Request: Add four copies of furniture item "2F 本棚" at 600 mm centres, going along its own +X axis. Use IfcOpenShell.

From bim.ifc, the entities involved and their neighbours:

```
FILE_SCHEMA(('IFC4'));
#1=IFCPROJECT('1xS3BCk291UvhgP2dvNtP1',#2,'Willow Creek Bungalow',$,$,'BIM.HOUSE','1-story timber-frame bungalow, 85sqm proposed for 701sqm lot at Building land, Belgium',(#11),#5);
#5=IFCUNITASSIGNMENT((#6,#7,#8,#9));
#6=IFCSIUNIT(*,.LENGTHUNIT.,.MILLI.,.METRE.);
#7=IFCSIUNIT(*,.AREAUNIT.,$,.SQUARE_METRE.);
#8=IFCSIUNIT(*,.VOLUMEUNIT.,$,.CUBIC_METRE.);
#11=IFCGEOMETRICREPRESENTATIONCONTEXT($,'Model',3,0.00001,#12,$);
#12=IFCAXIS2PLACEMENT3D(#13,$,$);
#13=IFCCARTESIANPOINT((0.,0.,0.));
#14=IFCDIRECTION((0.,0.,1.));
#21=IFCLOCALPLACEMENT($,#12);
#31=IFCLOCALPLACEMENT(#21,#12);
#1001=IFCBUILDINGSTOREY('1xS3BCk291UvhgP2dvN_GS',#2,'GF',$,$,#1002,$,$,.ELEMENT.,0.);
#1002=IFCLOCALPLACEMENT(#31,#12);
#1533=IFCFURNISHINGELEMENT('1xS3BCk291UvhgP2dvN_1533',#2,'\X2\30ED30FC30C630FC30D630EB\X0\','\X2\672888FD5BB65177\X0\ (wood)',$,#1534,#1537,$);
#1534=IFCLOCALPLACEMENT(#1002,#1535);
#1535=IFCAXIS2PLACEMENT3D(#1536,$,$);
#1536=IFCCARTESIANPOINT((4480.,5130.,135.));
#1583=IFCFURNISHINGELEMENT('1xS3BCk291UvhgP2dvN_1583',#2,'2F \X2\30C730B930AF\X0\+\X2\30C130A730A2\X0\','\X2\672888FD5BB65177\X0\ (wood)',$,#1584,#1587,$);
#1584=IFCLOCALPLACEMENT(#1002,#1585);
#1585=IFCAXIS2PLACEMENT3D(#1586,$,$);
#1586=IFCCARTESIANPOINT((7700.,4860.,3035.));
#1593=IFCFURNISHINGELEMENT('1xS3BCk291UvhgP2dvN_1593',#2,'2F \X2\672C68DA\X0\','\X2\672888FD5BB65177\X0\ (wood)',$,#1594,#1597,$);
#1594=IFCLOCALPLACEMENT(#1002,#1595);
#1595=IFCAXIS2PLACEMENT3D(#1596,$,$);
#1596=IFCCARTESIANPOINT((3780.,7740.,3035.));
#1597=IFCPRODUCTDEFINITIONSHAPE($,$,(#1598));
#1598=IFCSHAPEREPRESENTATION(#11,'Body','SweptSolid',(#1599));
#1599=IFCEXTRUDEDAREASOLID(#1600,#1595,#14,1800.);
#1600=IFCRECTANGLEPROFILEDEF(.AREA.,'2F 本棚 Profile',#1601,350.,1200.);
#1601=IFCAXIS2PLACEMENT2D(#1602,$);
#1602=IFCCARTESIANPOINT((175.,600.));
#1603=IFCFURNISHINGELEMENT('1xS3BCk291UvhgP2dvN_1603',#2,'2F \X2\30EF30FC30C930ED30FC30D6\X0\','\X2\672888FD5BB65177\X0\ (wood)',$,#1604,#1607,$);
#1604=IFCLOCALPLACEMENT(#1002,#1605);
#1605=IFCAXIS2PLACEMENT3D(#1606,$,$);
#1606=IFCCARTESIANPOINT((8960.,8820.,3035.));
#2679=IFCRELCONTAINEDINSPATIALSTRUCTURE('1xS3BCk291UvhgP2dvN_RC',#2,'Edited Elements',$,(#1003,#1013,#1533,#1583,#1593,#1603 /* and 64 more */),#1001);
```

```python
import ifcopenshell
import ifcopenshell.api.geometry
import ifcopenshell.api.root
import ifcopenshell.util.element
import ifcopenshell.util.placement
import ifcopenshell.util.unit

model = ifcopenshell.open("bim.ifc")
unit_scale = ifcopenshell.util.unit.calculate_unit_scale(model)


def reuse_history(source, copy):
    """copy_class also copies each property set's owner history, people and application; keep the originals."""
    for rel in copy.IsDefinedBy:
        if rel.is_a("IfcRelDefinesByProperties") and (history := rel.RelatingPropertyDefinition.OwnerHistory):
            rel.RelatingPropertyDefinition.OwnerHistory = source.OwnerHistory
            ifcopenshell.util.element.remove_deep2(model, history)


source = model.by_guid("1xS3BCk291UvhgP2dvN_1593")
base = ifcopenshell.util.placement.get_local_placement(source.ObjectPlacement)
step = base[:3, 0] * 0.6 / unit_scale

for i in range(1, 5):
    copy = ifcopenshell.api.root.copy_class(model, product=source)
    copy.Representation = ifcopenshell.util.element.copy_deep(
        model, source.Representation, exclude=["IfcGeometricRepresentationContext", "IfcRepresentationMap"]
    )
    reuse_history(source, copy)
    matrix = base.copy()
    matrix[:3, 3] += i * step
    print("added at", matrix[:3, 3].round(3) + 0.0)
    ifcopenshell.api.geometry.edit_object_placement(model, product=copy, matrix=matrix, is_si=False)

model.write("bim_v2.ifc")
```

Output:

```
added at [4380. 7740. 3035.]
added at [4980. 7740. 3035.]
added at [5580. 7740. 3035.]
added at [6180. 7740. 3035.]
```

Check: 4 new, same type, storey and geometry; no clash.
